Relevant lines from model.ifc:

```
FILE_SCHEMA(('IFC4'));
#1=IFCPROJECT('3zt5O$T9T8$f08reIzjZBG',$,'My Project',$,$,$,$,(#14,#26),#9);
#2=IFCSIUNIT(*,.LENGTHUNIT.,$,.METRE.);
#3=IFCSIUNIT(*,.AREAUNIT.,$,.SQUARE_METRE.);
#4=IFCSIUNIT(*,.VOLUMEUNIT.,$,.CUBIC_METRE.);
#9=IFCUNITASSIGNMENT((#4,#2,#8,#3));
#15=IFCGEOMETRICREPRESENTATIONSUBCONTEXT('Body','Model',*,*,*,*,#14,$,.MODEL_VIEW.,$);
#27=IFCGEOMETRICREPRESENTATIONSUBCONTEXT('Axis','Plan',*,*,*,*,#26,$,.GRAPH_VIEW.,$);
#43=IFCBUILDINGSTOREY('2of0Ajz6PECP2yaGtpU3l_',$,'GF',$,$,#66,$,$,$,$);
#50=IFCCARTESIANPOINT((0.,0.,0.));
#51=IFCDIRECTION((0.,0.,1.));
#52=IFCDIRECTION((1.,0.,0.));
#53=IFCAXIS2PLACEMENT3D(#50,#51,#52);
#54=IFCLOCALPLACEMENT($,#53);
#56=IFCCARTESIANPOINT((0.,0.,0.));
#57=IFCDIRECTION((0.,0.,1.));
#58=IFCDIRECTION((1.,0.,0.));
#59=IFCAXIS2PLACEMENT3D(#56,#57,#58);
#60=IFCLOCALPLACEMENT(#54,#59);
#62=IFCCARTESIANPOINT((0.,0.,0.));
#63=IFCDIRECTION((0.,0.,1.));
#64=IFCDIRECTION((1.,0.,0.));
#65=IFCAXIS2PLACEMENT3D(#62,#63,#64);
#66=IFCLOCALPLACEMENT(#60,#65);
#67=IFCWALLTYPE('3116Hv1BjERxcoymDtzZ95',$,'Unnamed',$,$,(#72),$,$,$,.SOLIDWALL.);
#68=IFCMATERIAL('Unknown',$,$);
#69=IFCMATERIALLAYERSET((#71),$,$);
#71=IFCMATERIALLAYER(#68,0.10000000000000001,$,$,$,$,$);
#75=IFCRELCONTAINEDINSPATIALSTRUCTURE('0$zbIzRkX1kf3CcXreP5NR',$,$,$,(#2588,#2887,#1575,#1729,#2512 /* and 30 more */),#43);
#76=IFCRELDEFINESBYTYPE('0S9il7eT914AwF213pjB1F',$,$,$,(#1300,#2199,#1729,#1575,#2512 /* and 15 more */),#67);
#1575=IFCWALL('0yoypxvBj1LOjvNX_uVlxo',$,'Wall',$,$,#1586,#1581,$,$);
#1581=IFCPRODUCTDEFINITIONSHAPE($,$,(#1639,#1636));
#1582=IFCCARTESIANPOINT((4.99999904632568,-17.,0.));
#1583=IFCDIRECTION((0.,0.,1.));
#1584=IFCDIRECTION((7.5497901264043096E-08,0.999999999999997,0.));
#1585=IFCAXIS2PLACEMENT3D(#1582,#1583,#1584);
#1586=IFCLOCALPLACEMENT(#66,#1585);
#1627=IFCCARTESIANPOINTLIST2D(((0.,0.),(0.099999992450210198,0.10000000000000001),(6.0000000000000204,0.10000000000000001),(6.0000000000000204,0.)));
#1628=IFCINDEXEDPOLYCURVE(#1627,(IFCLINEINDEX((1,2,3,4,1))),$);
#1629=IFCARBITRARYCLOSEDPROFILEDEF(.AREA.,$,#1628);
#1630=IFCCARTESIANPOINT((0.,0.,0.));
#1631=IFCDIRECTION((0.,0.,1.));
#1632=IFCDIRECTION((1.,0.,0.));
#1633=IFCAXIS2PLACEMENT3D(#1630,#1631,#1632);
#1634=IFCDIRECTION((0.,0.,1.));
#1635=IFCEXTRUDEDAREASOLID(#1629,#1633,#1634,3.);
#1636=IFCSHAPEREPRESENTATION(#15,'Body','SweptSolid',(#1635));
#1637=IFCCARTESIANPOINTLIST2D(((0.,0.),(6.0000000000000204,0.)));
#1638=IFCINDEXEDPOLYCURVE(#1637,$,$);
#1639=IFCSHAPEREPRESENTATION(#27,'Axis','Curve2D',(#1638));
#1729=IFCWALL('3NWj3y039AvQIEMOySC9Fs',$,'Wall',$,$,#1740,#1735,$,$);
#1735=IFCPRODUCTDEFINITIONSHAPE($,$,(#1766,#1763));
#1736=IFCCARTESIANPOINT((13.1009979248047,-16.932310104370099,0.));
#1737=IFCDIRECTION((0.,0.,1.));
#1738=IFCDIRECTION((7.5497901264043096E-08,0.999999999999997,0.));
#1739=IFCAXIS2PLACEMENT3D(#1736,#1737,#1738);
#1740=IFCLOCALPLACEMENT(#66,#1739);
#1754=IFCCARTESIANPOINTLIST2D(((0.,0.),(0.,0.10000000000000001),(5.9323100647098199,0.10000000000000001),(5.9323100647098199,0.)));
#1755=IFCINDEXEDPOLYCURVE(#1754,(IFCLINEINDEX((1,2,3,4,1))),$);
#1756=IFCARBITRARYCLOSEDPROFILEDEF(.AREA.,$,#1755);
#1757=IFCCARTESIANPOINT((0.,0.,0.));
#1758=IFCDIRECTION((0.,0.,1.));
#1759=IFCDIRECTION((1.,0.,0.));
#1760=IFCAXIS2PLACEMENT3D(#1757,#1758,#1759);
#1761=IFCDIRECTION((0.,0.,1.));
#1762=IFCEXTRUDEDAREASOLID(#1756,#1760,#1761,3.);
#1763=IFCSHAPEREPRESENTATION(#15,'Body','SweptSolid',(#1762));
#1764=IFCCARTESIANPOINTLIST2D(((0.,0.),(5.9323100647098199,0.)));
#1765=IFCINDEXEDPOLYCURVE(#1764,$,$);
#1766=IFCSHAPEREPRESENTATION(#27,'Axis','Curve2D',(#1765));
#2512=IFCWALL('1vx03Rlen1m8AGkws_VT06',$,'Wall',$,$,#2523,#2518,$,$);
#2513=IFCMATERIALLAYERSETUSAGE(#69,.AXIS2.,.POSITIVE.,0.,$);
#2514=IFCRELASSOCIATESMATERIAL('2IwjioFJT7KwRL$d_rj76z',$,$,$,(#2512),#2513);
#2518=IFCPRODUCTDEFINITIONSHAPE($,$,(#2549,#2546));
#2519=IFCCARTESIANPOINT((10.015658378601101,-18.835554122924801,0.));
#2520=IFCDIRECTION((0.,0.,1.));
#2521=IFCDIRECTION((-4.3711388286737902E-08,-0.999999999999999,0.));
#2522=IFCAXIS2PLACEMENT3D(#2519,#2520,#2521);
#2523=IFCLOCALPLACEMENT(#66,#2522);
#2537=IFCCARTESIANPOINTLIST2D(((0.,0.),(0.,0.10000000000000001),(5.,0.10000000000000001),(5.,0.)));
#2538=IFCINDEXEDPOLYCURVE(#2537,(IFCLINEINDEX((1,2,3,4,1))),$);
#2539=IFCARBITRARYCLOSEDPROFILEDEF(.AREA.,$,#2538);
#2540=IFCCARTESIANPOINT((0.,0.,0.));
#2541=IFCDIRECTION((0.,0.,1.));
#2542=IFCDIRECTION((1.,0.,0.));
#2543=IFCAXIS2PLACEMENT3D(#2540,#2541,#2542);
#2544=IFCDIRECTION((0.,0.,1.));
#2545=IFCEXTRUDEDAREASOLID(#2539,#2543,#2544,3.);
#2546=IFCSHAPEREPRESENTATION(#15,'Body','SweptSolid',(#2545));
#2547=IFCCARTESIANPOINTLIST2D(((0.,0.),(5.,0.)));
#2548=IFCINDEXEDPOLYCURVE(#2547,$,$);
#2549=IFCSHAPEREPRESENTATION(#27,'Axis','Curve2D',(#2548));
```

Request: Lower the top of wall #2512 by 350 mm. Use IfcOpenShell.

```python
import ifcopenshell
import ifcopenshell.geom
import ifcopenshell.util.representation
import ifcopenshell.util.shape

model = ifcopenshell.open("model.ifc")
settings = ifcopenshell.geom.settings()


def volume(element):
    """Net volume in cubic metres, openings subtracted."""
    shape = ifcopenshell.geom.create_shape(settings, element)
    return ifcopenshell.util.shape.get_volume(shape.geometry)


wall = model.by_id(2512)
before = volume(wall)

body = ifcopenshell.util.representation.get_representation(wall, "Model", "Body")
solid = body.Items[0]
old_height = solid.Depth
solid.Depth -= 0.35
after = volume(wall)

print(f"height {old_height:g} -> {solid.Depth:g}, volume {before:.3f} -> {after:.3f} m3")

model.write("model_v2.ifc")
```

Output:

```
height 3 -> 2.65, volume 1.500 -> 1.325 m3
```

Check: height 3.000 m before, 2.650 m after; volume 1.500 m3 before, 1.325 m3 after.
